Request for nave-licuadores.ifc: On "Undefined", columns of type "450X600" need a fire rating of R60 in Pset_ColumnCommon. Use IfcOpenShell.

First a look at what the model holds.

```python
import ifcopenshell
import ifcopenshell.util.element

model = ifcopenshell.open("nave-licuadores.ifc")
print(model.schema)
storey = next(s for s in model.by_type("IfcBuildingStorey") if s.Name == "Undefined")
columns = [e for e in ifcopenshell.util.element.get_decomposition(storey) if e.is_a("IfcColumn")]
seen = {}
for e in columns:
    element_type = ifcopenshell.util.element.get_type(e)
    key = (element_type.Name if element_type != e and element_type else None, ifcopenshell.util.element.get_pset(e, "Pset_ColumnCommon", "FireRating"))
    seen[key] = seen.get(key, 0) + 1
for (name, value), count in sorted(seen.items(), key=str):
    print(count, "x", name, "|", value)
```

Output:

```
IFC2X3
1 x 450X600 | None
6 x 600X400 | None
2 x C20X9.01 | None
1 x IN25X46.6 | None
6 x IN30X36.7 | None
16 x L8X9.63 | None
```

```python
import ifcopenshell
import ifcopenshell.api.pset
import ifcopenshell.util.element

model = ifcopenshell.open("nave-licuadores.ifc")

storey = next(s for s in model.by_type("IfcBuildingStorey") if s.Name == "Undefined")
columns = [e for e in ifcopenshell.util.element.get_decomposition(storey) if e.is_a("IfcColumn")]

count = 0
for e in columns:
    element_type = ifcopenshell.util.element.get_type(e)
    if element_type in (None, e) or element_type.Name != "450X600":
        continue
    # add_pset returns the element's existing set when there is one.
    pset = ifcopenshell.api.pset.add_pset(model, product=e, name="Pset_ColumnCommon")
    ifcopenshell.api.pset.edit_pset(model, pset=pset, properties={"FireRating": "R60"})
    count += 1

print(count, "columns updated")

model.write("nave-licuadores_rev.ifc")
```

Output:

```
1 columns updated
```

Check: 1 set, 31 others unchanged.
